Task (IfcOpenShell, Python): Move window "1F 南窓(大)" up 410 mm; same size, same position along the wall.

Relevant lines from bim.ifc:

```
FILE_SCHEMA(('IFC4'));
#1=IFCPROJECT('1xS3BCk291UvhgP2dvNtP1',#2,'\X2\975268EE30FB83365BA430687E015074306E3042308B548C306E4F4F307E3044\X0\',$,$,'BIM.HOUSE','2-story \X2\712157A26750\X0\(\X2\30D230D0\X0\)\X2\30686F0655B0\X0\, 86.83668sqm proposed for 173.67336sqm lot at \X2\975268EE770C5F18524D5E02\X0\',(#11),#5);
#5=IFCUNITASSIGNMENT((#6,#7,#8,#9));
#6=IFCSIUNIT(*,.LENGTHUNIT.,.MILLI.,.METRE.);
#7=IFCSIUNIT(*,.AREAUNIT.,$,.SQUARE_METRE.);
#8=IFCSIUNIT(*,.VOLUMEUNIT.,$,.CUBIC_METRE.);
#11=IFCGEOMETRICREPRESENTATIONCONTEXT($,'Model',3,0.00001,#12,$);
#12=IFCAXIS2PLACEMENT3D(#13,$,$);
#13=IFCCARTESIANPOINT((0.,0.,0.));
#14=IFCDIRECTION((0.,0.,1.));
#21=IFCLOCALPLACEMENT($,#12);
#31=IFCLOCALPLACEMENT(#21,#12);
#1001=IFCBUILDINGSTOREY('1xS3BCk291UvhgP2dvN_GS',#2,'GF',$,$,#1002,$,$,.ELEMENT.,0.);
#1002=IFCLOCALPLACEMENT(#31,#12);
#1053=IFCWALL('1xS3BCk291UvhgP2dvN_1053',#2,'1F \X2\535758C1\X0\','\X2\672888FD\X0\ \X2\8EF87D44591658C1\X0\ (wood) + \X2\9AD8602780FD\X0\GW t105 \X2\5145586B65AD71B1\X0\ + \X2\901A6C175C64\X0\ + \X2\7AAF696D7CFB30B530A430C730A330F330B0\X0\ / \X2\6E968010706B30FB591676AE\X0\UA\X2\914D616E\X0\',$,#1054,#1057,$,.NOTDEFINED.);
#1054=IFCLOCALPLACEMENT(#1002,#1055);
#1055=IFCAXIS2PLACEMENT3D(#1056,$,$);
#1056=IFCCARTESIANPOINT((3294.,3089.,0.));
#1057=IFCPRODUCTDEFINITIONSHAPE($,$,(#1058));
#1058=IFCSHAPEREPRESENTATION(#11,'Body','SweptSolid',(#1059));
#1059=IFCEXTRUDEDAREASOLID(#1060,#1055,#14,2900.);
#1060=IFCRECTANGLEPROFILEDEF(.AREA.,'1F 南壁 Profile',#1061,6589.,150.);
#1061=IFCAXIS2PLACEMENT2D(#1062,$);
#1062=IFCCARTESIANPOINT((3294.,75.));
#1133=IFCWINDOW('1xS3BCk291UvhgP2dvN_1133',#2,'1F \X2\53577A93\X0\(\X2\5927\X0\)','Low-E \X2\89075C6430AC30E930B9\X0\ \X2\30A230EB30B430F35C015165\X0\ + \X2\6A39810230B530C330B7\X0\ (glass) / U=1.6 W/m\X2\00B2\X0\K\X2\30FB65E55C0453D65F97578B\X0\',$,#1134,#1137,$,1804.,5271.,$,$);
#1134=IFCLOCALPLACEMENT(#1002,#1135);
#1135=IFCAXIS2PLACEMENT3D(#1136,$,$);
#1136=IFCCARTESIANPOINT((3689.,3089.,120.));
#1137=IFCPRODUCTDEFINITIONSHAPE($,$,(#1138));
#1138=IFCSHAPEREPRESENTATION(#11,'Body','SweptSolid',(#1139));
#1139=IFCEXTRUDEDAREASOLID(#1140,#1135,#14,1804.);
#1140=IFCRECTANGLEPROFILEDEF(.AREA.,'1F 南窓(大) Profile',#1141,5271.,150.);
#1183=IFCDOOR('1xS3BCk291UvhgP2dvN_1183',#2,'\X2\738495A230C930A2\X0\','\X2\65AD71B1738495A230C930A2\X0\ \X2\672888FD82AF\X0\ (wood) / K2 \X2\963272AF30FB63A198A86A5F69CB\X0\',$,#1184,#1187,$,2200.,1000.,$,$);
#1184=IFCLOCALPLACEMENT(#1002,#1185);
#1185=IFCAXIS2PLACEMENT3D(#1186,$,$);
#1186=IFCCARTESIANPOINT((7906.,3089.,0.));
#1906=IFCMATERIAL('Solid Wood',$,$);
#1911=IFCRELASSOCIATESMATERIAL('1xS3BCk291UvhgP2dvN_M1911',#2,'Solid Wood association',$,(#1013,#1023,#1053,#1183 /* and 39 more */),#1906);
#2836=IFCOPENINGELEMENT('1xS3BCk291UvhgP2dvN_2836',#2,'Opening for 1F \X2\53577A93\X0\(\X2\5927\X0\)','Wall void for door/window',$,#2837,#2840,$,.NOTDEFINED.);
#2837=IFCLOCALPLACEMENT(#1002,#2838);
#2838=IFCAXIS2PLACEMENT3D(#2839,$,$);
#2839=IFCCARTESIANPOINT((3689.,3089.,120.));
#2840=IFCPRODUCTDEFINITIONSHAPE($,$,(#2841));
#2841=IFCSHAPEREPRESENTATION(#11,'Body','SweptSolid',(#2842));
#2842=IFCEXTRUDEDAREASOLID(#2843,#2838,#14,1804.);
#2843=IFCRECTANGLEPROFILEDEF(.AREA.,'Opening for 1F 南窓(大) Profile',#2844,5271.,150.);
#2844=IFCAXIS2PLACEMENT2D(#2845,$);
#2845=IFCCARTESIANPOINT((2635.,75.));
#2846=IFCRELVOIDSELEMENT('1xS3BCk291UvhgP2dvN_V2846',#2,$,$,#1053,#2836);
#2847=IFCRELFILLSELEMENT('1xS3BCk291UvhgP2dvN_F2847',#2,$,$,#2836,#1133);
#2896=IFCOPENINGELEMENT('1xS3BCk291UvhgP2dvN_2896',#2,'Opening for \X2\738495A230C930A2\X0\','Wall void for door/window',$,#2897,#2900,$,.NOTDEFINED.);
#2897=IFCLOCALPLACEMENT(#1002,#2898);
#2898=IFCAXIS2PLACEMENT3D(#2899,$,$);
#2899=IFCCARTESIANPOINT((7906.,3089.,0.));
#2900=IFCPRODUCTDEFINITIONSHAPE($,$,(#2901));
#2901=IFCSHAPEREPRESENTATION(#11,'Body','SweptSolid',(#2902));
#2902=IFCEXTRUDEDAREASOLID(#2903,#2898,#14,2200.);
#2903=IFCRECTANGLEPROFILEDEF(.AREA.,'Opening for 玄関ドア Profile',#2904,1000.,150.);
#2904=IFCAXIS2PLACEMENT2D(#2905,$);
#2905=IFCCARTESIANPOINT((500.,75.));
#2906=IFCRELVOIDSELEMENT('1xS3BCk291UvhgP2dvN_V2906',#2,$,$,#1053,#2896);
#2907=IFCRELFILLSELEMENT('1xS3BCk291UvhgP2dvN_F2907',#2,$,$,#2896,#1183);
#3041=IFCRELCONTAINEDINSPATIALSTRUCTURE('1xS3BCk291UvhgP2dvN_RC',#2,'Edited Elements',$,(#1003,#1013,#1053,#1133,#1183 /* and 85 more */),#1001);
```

```python
import numpy as np
import ifcopenshell
import ifcopenshell.api.geometry
import ifcopenshell.util.placement
import ifcopenshell.util.unit

model = ifcopenshell.open("bim.ifc")
unit_scale = ifcopenshell.util.unit.calculate_unit_scale(model)

window = model.by_guid("1xS3BCk291UvhgP2dvN_1133")
opening = window.FillsVoids[0].RelatingOpeningElement
dz = 0.41 / unit_scale

shift = np.array([0.0, 0.0, dz])
# The window is not placed relative to its opening, so move both.
for product in (opening, window):
    matrix = ifcopenshell.util.placement.get_local_placement(product.ObjectPlacement)
    matrix[:3, 3] += shift
    ifcopenshell.api.geometry.edit_object_placement(model, product=product, matrix=matrix, is_si=False)

print(f"moved by {dz * unit_scale:+.3f} m")

model.write("bim_updated.ifc")
```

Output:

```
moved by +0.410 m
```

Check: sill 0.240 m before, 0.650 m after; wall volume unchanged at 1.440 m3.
